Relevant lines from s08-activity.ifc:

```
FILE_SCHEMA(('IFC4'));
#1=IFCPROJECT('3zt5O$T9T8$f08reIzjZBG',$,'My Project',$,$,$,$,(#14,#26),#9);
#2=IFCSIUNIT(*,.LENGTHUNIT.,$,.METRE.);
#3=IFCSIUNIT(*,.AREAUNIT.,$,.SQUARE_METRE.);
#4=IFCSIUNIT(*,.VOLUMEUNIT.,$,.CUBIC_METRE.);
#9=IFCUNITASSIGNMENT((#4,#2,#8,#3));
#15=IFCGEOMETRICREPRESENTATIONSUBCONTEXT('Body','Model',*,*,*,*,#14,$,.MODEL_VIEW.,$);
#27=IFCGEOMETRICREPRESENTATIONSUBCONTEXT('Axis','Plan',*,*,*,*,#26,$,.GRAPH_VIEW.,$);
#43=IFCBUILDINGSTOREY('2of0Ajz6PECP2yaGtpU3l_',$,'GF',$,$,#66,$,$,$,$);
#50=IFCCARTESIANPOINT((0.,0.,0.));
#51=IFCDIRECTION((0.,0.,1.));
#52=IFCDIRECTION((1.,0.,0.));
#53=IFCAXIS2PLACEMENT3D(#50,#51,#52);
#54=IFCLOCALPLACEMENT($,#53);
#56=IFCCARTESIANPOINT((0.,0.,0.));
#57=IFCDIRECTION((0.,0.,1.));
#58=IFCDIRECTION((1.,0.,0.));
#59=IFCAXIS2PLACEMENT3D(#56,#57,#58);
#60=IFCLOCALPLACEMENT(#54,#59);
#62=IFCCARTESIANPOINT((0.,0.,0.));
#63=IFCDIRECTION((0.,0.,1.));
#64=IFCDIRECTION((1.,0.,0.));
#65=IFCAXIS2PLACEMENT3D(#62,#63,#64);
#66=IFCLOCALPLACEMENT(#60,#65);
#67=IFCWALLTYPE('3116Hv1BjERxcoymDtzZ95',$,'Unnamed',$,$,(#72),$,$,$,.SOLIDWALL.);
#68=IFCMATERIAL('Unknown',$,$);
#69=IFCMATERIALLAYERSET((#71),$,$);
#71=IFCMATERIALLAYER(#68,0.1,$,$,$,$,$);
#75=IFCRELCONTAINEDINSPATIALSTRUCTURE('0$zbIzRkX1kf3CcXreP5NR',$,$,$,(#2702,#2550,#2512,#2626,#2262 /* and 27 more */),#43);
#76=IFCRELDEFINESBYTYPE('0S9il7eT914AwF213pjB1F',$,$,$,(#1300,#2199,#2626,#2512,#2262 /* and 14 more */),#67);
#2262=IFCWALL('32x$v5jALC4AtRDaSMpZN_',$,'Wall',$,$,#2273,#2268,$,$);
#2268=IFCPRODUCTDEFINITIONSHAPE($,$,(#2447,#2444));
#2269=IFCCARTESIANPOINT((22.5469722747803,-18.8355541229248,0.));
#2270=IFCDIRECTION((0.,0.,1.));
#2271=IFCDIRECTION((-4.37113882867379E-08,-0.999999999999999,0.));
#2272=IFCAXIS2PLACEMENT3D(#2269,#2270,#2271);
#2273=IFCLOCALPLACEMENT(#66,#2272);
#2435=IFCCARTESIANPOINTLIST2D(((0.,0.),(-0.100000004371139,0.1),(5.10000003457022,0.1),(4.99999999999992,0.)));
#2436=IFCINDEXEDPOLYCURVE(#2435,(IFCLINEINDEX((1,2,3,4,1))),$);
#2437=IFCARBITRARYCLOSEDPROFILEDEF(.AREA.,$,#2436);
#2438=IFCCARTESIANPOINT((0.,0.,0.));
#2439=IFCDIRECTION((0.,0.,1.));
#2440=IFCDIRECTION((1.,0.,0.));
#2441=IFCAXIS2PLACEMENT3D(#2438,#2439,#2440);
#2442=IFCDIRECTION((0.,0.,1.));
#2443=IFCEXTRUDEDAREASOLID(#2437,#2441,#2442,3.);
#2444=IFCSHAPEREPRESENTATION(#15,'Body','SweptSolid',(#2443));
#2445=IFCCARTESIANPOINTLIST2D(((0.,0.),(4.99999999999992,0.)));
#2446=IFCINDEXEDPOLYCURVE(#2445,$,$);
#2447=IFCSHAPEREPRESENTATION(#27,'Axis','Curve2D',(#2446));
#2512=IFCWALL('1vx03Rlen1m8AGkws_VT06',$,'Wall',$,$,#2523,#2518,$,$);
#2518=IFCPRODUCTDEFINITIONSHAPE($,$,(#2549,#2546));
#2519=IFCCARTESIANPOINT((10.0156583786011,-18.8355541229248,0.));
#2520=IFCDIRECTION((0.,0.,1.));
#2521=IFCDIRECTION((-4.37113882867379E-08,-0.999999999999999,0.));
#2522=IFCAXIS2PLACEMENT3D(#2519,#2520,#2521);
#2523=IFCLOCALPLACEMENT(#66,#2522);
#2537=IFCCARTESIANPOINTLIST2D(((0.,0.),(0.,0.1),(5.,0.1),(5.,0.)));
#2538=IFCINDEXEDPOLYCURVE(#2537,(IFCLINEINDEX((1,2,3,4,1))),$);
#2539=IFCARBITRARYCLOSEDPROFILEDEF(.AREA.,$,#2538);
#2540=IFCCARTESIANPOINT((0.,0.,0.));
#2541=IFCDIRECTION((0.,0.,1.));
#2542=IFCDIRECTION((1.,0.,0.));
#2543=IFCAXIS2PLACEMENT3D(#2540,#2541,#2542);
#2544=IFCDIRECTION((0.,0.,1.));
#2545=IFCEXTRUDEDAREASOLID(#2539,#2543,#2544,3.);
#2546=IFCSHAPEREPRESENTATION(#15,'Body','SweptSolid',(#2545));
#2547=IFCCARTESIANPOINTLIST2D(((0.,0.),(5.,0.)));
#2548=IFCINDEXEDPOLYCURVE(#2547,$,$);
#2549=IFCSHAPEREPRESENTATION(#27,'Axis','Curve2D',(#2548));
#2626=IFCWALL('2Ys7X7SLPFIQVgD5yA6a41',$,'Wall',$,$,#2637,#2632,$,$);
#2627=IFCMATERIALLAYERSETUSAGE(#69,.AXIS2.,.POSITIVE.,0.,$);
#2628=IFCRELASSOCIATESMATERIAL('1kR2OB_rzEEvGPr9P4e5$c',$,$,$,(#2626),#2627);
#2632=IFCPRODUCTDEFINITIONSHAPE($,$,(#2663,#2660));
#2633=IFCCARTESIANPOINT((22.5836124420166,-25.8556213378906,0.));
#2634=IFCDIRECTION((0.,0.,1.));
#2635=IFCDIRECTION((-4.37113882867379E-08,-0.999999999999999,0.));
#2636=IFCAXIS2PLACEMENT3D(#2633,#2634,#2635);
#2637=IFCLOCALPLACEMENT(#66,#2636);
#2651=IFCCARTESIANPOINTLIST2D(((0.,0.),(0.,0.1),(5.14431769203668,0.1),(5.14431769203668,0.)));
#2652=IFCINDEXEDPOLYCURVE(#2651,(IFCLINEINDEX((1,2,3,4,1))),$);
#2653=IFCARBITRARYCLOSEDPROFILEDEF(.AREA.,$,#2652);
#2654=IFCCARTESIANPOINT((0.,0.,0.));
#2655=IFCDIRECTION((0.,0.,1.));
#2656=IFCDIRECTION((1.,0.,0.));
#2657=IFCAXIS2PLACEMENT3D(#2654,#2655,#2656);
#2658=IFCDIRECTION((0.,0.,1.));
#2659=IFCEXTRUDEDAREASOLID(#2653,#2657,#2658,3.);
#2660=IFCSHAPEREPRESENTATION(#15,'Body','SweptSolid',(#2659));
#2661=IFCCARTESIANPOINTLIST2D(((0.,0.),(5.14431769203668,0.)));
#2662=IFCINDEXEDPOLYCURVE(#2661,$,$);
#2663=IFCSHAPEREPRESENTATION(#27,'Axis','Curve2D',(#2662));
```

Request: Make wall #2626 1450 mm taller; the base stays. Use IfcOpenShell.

```python
import ifcopenshell
import ifcopenshell.geom
import ifcopenshell.util.representation
import ifcopenshell.util.shape
import ifcopenshell.util.unit

model = ifcopenshell.open("s08-activity.ifc")
unit_scale = ifcopenshell.util.unit.calculate_unit_scale(model)
settings = ifcopenshell.geom.settings()


def volume(element):
    """Net volume in cubic metres, openings subtracted."""
    shape = ifcopenshell.geom.create_shape(settings, element)
    return ifcopenshell.util.shape.get_volume(shape.geometry)


wall = model.by_id(2626)
before = volume(wall)

body = ifcopenshell.util.representation.get_representation(wall, "Model", "Body")
solid = body.Items[0]
old_height = solid.Depth
solid.Depth += 1.45 / unit_scale
after = volume(wall)

print(f"height {old_height:g} -> {solid.Depth:g}, volume {before:.3f} -> {after:.3f} m3")

model.write("s08-activity_updated.ifc")
```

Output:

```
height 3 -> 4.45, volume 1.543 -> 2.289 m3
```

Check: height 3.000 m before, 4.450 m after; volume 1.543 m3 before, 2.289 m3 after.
